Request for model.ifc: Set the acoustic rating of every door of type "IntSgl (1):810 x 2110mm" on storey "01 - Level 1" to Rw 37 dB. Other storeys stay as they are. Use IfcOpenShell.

First a look at what the model holds.

```python
import ifcopenshell
import ifcopenshell.util.element

model = ifcopenshell.open("model.ifc")
print(model.schema)
storey = next(s for s in model.by_type("IfcBuildingStorey") if s.Name == "01 - Level 1")
doors = [e for e in ifcopenshell.util.element.get_decomposition(storey) if e.is_a("IfcDoor")]
seen = {}
for e in doors:
    element_type = ifcopenshell.util.element.get_type(e)
    key = (element_type.Name if element_type != e and element_type else None, ifcopenshell.util.element.get_pset(e, "Pset_DoorCommon", "AcousticRating"))
    seen[key] = seen.get(key, 0) + 1
for (name, value), count in sorted(seen.items(), key=str):
    print(count, "x", name, "|", value)
```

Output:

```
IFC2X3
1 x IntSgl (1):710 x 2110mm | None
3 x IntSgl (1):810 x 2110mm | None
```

```python
import ifcopenshell
import ifcopenshell.api.pset
import ifcopenshell.util.element

model = ifcopenshell.open("model.ifc")

storey = next(s for s in model.by_type("IfcBuildingStorey") if s.Name == "01 - Level 1")
doors = [e for e in ifcopenshell.util.element.get_decomposition(storey) if e.is_a("IfcDoor")]

count = 0
for e in doors:
    element_type = ifcopenshell.util.element.get_type(e)
    if element_type in (None, e) or element_type.Name != "IntSgl (1):810 x 2110mm":
        continue
    # add_pset returns the element's existing set when there is one.
    pset = ifcopenshell.api.pset.add_pset(model, product=e, name="Pset_DoorCommon")
    ifcopenshell.api.pset.edit_pset(model, pset=pset, properties={"AcousticRating": "Rw 37 dB"})
    count += 1

print(count, "doors updated")

model.write("model_rev.ifc")
```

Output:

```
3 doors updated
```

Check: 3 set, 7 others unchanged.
